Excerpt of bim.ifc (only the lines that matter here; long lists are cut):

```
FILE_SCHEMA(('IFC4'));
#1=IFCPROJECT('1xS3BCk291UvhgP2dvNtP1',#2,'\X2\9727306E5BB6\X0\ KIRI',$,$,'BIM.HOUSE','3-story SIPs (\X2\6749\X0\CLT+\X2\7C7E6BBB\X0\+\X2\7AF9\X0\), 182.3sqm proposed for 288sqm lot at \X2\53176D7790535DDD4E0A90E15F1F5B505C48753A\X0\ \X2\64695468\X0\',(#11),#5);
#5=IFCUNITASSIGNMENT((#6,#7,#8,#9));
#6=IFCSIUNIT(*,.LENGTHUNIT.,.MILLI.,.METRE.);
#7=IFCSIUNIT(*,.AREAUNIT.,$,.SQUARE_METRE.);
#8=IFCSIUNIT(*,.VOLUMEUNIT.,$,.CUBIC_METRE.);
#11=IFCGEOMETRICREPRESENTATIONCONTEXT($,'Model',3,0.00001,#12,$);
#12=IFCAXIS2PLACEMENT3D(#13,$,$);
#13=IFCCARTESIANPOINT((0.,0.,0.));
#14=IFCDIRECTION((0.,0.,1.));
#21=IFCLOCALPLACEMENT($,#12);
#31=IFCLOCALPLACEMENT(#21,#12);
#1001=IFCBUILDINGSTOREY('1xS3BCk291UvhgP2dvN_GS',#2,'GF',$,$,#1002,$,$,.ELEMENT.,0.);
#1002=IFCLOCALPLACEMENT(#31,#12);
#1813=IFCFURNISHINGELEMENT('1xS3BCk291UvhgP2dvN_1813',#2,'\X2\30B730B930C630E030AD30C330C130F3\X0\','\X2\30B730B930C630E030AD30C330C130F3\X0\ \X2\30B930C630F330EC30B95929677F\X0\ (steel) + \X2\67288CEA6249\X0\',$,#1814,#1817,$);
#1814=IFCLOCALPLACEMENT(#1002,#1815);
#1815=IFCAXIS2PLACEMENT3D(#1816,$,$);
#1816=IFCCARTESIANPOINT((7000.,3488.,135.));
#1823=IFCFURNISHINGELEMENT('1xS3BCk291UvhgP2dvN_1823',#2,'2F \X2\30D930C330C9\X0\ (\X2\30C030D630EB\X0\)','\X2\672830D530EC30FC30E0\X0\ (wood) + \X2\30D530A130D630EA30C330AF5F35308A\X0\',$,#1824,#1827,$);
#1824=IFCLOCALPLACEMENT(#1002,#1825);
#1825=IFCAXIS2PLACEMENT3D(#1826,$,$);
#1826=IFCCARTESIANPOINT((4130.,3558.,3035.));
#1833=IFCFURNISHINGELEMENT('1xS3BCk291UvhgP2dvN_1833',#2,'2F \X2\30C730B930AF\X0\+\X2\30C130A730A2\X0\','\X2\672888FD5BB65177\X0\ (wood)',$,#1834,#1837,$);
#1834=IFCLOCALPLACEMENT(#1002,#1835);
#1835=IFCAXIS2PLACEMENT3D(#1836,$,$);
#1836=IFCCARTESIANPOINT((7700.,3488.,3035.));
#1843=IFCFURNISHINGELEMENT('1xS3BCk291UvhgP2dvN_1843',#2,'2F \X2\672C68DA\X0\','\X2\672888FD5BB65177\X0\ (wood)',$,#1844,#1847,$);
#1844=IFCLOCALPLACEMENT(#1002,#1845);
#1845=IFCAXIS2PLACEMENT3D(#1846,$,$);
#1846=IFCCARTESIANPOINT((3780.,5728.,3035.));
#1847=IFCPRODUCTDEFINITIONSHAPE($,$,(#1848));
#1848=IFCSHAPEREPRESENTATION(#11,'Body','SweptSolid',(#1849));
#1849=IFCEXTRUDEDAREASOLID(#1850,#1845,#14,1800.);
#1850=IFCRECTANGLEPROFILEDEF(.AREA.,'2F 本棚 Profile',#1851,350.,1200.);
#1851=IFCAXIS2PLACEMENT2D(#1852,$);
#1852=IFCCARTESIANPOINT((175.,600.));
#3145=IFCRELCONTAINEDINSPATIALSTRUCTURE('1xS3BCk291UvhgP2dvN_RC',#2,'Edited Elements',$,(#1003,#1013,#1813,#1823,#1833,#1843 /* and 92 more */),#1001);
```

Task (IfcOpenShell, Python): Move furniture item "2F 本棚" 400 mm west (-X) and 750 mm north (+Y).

```python
import ifcopenshell
import ifcopenshell.api.geometry
import ifcopenshell.util.placement
import ifcopenshell.util.unit

model = ifcopenshell.open("bim.ifc")
unit_scale = ifcopenshell.util.unit.calculate_unit_scale(model)

item = model.by_guid("1xS3BCk291UvhgP2dvN_1843")
matrix = ifcopenshell.util.placement.get_local_placement(item.ObjectPlacement)
matrix[0, 3] -= 0.4 / unit_scale
matrix[1, 3] += 0.75 / unit_scale
ifcopenshell.api.geometry.edit_object_placement(model, product=item, matrix=matrix, is_si=False)

print(ifcopenshell.util.placement.get_local_placement(item.ObjectPlacement).round(3) + 0.0)

model.write("bim_edited.ifc")
```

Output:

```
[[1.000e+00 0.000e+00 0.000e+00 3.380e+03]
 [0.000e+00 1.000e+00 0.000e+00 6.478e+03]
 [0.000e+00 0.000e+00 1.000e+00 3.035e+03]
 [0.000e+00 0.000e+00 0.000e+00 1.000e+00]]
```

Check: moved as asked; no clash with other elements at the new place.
